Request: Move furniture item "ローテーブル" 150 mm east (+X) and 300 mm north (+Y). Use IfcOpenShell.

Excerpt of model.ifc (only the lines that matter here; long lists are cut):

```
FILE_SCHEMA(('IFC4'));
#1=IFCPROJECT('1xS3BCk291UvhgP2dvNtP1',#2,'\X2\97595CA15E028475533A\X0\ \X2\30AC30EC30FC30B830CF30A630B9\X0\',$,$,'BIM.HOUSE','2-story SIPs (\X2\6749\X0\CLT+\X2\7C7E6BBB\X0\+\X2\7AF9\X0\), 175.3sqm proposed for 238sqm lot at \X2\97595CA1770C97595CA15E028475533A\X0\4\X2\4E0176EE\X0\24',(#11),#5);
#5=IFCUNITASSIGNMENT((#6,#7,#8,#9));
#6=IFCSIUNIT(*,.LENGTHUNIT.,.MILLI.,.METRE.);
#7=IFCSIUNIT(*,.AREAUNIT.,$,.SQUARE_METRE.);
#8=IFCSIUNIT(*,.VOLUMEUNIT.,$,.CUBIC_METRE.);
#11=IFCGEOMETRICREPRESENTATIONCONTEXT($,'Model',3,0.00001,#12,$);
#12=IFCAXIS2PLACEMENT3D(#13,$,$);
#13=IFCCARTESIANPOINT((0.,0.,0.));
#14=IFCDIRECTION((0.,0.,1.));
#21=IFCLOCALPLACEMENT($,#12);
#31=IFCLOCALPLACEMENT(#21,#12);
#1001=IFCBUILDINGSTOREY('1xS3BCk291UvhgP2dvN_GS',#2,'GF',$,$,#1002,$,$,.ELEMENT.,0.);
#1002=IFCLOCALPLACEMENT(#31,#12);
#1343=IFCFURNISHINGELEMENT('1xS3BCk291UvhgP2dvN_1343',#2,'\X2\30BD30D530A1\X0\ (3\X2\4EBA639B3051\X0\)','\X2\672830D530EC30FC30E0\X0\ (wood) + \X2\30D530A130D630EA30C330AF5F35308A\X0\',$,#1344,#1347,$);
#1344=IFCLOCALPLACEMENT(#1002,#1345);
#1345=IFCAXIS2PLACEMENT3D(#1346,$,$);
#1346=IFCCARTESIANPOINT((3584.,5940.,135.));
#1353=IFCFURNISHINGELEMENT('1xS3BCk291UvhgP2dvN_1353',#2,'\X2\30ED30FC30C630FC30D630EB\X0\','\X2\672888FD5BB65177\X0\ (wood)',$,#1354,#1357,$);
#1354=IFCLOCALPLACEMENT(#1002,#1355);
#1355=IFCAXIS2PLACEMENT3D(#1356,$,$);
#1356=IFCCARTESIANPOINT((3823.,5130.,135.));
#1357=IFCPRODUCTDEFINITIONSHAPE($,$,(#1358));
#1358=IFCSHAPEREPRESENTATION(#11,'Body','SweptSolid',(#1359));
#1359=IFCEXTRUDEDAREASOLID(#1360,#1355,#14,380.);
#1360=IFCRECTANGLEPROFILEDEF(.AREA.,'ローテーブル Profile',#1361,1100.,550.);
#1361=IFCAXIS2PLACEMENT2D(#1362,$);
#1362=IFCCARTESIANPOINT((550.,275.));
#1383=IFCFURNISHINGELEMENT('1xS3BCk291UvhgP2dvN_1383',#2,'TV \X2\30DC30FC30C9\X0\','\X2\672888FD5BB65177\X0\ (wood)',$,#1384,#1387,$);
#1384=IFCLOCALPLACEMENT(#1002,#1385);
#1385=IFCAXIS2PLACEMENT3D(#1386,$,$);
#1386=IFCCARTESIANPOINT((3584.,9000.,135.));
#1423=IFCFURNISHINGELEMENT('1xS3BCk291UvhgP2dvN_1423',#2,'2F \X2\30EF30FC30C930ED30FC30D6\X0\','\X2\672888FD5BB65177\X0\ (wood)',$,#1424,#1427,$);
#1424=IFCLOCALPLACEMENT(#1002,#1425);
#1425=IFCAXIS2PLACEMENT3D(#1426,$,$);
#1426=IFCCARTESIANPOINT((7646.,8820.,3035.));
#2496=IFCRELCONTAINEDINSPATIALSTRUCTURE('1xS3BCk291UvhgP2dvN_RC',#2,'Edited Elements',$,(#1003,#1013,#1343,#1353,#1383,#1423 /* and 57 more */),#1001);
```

```python
import ifcopenshell
import ifcopenshell.api.geometry
import ifcopenshell.util.placement

model = ifcopenshell.open("model.ifc")

item = model.by_guid("1xS3BCk291UvhgP2dvN_1353")
matrix = ifcopenshell.util.placement.get_local_placement(item.ObjectPlacement)
matrix[0, 3] += 150.0
matrix[1, 3] += 300.0
ifcopenshell.api.geometry.edit_object_placement(model, product=item, matrix=matrix, is_si=False)

print(ifcopenshell.util.placement.get_local_placement(item.ObjectPlacement).round(3) + 0.0)

model.write("model_updated.ifc")
```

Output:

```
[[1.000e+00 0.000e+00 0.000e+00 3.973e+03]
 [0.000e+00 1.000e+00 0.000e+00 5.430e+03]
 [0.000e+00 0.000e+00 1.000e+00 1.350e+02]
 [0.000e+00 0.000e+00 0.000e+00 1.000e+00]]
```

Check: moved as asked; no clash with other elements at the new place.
